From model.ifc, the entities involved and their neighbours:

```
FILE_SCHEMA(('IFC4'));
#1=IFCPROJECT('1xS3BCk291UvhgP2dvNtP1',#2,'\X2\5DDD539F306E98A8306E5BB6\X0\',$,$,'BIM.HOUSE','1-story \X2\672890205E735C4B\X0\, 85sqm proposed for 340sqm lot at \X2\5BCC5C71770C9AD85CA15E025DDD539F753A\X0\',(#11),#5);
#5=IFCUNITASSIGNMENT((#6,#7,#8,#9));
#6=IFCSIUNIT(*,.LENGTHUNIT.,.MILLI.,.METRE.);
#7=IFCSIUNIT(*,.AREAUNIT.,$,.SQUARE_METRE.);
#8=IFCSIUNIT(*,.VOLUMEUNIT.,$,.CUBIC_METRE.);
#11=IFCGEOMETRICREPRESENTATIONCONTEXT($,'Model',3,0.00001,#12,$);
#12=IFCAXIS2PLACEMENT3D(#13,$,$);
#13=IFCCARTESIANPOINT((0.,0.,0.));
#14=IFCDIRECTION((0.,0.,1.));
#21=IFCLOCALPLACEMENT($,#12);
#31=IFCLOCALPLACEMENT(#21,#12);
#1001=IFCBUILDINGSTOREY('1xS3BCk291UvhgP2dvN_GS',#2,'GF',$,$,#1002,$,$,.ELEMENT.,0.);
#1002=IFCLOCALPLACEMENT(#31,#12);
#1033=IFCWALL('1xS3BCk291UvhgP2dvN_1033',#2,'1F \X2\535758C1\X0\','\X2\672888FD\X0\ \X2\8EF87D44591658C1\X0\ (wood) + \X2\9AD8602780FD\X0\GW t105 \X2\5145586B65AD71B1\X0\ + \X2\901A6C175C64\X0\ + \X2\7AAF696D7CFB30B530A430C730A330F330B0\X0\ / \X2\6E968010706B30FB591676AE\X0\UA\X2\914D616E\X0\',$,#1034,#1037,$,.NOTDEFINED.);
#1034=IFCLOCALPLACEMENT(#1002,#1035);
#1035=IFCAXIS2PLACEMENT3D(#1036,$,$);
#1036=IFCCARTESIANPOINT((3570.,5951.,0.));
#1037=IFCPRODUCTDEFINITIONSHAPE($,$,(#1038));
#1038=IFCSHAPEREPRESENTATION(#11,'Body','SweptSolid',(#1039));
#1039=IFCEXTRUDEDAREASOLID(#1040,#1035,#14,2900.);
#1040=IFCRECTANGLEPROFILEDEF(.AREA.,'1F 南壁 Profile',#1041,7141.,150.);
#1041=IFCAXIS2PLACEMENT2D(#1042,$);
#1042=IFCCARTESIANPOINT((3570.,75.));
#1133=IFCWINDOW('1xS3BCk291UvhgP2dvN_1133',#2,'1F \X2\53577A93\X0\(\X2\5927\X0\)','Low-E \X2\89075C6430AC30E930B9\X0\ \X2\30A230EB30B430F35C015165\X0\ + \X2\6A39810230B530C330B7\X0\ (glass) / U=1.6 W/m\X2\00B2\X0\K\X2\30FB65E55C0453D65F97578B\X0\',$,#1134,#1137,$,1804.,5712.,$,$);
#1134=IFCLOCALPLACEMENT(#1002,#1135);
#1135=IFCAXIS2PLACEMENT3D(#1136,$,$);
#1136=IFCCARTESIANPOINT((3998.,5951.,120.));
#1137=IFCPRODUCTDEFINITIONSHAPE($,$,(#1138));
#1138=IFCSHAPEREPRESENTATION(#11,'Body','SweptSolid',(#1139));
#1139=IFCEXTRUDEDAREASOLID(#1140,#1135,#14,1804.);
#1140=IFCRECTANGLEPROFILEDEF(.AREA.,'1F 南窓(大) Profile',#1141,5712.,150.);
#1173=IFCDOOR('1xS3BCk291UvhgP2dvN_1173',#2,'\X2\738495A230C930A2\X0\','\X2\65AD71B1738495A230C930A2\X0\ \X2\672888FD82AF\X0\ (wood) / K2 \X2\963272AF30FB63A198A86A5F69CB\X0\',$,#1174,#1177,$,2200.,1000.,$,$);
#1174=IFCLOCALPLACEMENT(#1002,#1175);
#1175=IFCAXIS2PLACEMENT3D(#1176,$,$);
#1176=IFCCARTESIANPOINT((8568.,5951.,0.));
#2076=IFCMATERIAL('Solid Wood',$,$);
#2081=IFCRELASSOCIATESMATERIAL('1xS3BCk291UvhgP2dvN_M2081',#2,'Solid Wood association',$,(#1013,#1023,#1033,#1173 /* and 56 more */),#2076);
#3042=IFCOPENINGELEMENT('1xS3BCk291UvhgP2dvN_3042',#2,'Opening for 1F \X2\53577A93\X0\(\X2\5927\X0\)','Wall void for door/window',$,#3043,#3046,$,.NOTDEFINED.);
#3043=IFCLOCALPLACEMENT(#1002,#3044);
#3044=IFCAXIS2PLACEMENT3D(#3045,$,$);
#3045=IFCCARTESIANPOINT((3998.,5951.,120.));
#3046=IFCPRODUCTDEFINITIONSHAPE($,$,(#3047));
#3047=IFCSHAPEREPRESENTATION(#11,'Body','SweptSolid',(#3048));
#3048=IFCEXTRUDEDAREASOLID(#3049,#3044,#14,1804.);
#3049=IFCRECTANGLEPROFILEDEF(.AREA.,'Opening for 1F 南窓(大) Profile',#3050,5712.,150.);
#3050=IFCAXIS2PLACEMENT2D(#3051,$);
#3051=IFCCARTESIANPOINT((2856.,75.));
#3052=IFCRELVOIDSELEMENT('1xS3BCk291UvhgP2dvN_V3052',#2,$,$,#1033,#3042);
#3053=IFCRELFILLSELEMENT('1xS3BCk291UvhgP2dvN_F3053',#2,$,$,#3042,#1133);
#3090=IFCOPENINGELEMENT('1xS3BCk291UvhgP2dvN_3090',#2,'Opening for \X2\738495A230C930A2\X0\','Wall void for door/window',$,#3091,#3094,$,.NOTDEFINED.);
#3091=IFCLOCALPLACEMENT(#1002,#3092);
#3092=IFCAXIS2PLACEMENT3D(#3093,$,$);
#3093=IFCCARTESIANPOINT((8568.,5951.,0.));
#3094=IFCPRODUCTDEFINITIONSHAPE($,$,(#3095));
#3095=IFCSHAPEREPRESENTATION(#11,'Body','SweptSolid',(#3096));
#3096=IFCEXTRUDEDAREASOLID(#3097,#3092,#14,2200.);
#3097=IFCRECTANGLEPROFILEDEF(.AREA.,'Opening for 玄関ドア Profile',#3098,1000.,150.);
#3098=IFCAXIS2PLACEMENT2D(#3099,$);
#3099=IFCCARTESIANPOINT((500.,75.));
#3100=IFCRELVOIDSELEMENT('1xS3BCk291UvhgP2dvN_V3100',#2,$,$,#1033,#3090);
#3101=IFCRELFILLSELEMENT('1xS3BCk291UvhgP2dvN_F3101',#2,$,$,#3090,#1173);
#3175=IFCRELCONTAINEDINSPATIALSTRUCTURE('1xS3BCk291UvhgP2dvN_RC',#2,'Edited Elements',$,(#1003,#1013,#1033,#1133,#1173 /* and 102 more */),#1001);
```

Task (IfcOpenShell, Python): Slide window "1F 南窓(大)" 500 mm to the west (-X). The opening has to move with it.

```python
import ifcopenshell
import ifcopenshell.api.geometry
import ifcopenshell.util.placement
import ifcopenshell.util.unit

model = ifcopenshell.open("model.ifc")
unit_scale = ifcopenshell.util.unit.calculate_unit_scale(model)

window = model.by_guid("1xS3BCk291UvhgP2dvN_1133")
opening = window.FillsVoids[0].RelatingOpeningElement
wall = opening.VoidsElements[0].RelatingBuildingElement

wall_matrix = ifcopenshell.util.placement.get_local_placement(wall.ObjectPlacement)
shift = wall_matrix[:3, 0] * -0.5 / unit_scale
before = ifcopenshell.util.placement.get_local_placement(window.ObjectPlacement)[:3, 3].copy()

# The window is not placed relative to its opening, so move both.
for product in (opening, window):
    matrix = ifcopenshell.util.placement.get_local_placement(product.ObjectPlacement)
    matrix[:3, 3] += shift
    ifcopenshell.api.geometry.edit_object_placement(model, product=product, matrix=matrix, is_si=False)

after = ifcopenshell.util.placement.get_local_placement(window.ObjectPlacement)[:3, 3]
print("window moved by", (after - before).round(3) + 0.0)

model.write("model_edited.ifc")
```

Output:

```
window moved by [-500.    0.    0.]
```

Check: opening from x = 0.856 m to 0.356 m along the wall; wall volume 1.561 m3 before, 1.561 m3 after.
